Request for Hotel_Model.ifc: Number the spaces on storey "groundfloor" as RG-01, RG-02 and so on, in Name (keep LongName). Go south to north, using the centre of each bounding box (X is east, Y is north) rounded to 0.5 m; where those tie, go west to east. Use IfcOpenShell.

First a look at what the model holds.

```python
import ifcopenshell
import ifcopenshell.util.element
import ifcopenshell.util.placement

model = ifcopenshell.open("Hotel_Model.ifc")
print(model.schema)
storey = next(s for s in model.by_type("IfcBuildingStorey") if s.Name == "groundfloor")
spaces = [e for e in ifcopenshell.util.element.get_decomposition(storey) if e.is_a("IfcSpace")]
for e in sorted(spaces, key=lambda e: e.id()):
    origin = ifcopenshell.util.placement.get_local_placement(e.ObjectPlacement)[:3, 3]
    print(e.id(), e.Name, e.LongName, origin.round(2) + 0.0, sep=" | ")
```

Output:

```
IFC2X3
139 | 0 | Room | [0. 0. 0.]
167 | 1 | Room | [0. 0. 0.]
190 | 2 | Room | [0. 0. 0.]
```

```python
import ifcopenshell
import ifcopenshell.geom
import ifcopenshell.util.element
import ifcopenshell.util.shape

model = ifcopenshell.open("Hotel_Model.ifc")
settings = ifcopenshell.geom.settings()
settings.set("use-world-coords", True)


def centre(element):
    shape = ifcopenshell.geom.create_shape(settings, element)
    return ifcopenshell.util.shape.get_bbox_centroid(shape.geometry)


storey = next(s for s in model.by_type("IfcBuildingStorey") if s.Name == "groundfloor")
spaces = [e for e in ifcopenshell.util.element.get_decomposition(storey) if e.is_a("IfcSpace")]

# Insertion points can sit at a corner or the storey origin, so sort by the geometry (in metres).
centres = {e: centre(e) for e in spaces}
spaces.sort(key=lambda e: (round(centres[e][1] / 0.5), centres[e][0]))

for i, e in enumerate(spaces, start=1):
    number = f"RG-{i:02d}"
    e.Name = number
    print(e.id(), number)

model.write("Hotel_Model-out.ifc")
```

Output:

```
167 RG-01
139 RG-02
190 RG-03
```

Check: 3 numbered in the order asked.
